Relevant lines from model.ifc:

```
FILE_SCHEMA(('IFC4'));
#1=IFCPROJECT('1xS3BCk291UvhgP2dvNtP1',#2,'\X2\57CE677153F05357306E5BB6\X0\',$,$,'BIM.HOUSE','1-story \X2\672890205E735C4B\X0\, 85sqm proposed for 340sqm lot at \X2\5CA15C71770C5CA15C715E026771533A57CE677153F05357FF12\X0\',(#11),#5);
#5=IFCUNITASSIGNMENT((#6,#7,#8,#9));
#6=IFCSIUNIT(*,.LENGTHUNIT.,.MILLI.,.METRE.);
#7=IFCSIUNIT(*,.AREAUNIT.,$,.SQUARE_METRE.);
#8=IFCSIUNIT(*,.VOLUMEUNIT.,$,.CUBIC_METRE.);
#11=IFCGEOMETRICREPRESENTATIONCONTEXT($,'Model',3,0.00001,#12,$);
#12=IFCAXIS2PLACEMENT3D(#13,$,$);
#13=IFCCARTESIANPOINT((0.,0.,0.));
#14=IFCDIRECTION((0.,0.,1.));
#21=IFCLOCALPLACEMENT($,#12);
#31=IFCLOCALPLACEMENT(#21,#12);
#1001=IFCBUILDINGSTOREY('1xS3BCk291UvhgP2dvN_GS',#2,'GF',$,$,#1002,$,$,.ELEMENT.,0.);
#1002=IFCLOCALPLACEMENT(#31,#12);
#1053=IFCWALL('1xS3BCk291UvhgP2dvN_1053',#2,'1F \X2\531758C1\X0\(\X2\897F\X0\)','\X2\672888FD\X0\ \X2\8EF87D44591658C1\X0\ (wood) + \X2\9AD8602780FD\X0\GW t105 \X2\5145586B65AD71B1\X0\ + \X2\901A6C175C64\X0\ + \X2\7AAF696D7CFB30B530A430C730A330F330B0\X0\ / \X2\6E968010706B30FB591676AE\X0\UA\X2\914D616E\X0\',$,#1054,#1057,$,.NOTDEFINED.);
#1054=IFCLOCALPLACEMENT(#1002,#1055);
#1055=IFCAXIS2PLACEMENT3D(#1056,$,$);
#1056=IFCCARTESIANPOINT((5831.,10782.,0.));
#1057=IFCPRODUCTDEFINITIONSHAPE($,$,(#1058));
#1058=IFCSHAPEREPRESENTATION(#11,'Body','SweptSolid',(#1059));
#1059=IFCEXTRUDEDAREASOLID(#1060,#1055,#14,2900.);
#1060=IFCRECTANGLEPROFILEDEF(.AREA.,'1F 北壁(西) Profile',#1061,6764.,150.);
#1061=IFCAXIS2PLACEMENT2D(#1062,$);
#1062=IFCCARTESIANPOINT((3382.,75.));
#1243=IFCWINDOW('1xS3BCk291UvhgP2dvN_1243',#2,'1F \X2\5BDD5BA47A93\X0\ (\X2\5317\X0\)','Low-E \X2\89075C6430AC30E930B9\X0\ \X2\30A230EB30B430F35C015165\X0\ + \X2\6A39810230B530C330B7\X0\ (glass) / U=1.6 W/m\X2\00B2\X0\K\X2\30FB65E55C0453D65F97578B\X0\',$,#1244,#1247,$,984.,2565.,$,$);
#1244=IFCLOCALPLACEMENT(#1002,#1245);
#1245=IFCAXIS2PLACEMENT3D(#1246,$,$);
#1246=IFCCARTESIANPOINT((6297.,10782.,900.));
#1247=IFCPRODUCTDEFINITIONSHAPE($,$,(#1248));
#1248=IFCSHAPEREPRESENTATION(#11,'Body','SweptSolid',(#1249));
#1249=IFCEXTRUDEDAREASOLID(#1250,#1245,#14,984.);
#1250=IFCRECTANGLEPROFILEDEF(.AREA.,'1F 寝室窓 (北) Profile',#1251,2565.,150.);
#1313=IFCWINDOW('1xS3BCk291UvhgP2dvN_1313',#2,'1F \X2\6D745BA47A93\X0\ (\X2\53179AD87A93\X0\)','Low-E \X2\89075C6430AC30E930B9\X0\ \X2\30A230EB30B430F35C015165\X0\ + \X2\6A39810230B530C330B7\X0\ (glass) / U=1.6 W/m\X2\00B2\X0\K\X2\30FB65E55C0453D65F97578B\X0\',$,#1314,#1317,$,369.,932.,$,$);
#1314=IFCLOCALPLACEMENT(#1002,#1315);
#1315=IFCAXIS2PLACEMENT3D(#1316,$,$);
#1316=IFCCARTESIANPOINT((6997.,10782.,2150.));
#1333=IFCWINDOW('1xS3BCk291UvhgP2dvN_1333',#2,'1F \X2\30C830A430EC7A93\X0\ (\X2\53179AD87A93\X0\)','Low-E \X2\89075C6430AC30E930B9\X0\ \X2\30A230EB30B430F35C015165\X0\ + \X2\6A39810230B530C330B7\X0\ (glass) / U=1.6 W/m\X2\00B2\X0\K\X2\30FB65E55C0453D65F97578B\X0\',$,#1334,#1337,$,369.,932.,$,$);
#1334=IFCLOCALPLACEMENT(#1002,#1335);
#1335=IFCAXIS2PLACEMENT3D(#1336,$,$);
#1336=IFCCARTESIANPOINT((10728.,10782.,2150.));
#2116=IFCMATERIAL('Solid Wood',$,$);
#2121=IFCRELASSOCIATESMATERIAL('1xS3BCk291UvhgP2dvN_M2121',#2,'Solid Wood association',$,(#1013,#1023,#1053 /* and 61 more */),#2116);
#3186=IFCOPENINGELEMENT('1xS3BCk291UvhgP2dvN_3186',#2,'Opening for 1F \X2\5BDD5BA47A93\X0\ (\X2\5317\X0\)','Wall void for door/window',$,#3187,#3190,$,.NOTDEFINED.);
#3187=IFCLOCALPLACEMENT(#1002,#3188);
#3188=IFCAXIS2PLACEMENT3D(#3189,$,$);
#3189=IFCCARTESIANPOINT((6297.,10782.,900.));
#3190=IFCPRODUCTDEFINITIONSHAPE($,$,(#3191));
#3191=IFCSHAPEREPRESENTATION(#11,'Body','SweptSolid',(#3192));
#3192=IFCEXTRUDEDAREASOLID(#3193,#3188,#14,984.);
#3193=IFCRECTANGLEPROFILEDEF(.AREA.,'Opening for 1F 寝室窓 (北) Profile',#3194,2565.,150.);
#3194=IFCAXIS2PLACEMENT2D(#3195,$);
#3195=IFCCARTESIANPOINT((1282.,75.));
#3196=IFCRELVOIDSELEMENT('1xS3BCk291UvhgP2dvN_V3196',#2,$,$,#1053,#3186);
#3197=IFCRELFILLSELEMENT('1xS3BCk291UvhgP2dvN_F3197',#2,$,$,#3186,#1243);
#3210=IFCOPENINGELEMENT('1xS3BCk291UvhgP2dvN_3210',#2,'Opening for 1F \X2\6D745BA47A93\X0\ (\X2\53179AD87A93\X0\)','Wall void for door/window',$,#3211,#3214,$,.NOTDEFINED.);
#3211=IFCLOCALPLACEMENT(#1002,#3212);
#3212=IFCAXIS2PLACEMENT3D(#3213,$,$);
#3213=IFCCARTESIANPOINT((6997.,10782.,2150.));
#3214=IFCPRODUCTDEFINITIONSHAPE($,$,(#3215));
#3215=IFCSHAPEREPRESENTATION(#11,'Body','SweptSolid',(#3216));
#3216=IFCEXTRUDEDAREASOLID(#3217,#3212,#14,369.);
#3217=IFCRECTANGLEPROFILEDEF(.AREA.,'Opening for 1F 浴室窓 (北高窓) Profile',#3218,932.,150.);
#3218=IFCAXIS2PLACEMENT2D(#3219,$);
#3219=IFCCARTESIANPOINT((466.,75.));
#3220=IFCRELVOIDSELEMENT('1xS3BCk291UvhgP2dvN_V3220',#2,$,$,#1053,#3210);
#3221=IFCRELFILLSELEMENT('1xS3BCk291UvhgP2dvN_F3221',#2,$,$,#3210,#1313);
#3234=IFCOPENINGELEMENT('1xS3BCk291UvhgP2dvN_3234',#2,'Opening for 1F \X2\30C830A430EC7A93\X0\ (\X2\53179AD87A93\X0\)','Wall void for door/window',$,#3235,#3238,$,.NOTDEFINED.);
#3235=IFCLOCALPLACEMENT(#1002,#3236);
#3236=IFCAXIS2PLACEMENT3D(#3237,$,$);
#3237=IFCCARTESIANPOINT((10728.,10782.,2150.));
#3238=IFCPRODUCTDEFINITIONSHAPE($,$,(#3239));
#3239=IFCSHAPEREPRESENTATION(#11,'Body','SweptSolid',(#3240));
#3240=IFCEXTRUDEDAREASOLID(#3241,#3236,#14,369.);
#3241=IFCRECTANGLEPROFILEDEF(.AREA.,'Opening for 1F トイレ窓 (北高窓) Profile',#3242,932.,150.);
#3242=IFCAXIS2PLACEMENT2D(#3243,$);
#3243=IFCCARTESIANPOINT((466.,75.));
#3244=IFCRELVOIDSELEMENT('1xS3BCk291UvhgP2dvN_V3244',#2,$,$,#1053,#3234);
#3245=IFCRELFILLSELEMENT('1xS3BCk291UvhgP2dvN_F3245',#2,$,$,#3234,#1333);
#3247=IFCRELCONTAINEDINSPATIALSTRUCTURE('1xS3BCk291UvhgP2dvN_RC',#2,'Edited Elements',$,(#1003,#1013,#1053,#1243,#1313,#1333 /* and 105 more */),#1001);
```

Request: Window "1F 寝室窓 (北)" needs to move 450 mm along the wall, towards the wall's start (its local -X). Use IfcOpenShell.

```python
import ifcopenshell
import ifcopenshell.api.geometry
import ifcopenshell.util.placement

model = ifcopenshell.open("model.ifc")

window = model.by_guid("1xS3BCk291UvhgP2dvN_1243")
opening = window.FillsVoids[0].RelatingOpeningElement
wall = opening.VoidsElements[0].RelatingBuildingElement

wall_matrix = ifcopenshell.util.placement.get_local_placement(wall.ObjectPlacement)
shift = wall_matrix[:3, 0] * -450.0
before = ifcopenshell.util.placement.get_local_placement(window.ObjectPlacement)[:3, 3].copy()

# The window is not placed relative to its opening, so move both.
for product in (opening, window):
    matrix = ifcopenshell.util.placement.get_local_placement(product.ObjectPlacement)
    matrix[:3, 3] += shift
    ifcopenshell.api.geometry.edit_object_placement(model, product=product, matrix=matrix, is_si=False)

after = ifcopenshell.util.placement.get_local_placement(window.ObjectPlacement)[:3, 3]
print("window moved by", (after - before).round(3) + 0.0)

model.write("model_rev.ifc")
```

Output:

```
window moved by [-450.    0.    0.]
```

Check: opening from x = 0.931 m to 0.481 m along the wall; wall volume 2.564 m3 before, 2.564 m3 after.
